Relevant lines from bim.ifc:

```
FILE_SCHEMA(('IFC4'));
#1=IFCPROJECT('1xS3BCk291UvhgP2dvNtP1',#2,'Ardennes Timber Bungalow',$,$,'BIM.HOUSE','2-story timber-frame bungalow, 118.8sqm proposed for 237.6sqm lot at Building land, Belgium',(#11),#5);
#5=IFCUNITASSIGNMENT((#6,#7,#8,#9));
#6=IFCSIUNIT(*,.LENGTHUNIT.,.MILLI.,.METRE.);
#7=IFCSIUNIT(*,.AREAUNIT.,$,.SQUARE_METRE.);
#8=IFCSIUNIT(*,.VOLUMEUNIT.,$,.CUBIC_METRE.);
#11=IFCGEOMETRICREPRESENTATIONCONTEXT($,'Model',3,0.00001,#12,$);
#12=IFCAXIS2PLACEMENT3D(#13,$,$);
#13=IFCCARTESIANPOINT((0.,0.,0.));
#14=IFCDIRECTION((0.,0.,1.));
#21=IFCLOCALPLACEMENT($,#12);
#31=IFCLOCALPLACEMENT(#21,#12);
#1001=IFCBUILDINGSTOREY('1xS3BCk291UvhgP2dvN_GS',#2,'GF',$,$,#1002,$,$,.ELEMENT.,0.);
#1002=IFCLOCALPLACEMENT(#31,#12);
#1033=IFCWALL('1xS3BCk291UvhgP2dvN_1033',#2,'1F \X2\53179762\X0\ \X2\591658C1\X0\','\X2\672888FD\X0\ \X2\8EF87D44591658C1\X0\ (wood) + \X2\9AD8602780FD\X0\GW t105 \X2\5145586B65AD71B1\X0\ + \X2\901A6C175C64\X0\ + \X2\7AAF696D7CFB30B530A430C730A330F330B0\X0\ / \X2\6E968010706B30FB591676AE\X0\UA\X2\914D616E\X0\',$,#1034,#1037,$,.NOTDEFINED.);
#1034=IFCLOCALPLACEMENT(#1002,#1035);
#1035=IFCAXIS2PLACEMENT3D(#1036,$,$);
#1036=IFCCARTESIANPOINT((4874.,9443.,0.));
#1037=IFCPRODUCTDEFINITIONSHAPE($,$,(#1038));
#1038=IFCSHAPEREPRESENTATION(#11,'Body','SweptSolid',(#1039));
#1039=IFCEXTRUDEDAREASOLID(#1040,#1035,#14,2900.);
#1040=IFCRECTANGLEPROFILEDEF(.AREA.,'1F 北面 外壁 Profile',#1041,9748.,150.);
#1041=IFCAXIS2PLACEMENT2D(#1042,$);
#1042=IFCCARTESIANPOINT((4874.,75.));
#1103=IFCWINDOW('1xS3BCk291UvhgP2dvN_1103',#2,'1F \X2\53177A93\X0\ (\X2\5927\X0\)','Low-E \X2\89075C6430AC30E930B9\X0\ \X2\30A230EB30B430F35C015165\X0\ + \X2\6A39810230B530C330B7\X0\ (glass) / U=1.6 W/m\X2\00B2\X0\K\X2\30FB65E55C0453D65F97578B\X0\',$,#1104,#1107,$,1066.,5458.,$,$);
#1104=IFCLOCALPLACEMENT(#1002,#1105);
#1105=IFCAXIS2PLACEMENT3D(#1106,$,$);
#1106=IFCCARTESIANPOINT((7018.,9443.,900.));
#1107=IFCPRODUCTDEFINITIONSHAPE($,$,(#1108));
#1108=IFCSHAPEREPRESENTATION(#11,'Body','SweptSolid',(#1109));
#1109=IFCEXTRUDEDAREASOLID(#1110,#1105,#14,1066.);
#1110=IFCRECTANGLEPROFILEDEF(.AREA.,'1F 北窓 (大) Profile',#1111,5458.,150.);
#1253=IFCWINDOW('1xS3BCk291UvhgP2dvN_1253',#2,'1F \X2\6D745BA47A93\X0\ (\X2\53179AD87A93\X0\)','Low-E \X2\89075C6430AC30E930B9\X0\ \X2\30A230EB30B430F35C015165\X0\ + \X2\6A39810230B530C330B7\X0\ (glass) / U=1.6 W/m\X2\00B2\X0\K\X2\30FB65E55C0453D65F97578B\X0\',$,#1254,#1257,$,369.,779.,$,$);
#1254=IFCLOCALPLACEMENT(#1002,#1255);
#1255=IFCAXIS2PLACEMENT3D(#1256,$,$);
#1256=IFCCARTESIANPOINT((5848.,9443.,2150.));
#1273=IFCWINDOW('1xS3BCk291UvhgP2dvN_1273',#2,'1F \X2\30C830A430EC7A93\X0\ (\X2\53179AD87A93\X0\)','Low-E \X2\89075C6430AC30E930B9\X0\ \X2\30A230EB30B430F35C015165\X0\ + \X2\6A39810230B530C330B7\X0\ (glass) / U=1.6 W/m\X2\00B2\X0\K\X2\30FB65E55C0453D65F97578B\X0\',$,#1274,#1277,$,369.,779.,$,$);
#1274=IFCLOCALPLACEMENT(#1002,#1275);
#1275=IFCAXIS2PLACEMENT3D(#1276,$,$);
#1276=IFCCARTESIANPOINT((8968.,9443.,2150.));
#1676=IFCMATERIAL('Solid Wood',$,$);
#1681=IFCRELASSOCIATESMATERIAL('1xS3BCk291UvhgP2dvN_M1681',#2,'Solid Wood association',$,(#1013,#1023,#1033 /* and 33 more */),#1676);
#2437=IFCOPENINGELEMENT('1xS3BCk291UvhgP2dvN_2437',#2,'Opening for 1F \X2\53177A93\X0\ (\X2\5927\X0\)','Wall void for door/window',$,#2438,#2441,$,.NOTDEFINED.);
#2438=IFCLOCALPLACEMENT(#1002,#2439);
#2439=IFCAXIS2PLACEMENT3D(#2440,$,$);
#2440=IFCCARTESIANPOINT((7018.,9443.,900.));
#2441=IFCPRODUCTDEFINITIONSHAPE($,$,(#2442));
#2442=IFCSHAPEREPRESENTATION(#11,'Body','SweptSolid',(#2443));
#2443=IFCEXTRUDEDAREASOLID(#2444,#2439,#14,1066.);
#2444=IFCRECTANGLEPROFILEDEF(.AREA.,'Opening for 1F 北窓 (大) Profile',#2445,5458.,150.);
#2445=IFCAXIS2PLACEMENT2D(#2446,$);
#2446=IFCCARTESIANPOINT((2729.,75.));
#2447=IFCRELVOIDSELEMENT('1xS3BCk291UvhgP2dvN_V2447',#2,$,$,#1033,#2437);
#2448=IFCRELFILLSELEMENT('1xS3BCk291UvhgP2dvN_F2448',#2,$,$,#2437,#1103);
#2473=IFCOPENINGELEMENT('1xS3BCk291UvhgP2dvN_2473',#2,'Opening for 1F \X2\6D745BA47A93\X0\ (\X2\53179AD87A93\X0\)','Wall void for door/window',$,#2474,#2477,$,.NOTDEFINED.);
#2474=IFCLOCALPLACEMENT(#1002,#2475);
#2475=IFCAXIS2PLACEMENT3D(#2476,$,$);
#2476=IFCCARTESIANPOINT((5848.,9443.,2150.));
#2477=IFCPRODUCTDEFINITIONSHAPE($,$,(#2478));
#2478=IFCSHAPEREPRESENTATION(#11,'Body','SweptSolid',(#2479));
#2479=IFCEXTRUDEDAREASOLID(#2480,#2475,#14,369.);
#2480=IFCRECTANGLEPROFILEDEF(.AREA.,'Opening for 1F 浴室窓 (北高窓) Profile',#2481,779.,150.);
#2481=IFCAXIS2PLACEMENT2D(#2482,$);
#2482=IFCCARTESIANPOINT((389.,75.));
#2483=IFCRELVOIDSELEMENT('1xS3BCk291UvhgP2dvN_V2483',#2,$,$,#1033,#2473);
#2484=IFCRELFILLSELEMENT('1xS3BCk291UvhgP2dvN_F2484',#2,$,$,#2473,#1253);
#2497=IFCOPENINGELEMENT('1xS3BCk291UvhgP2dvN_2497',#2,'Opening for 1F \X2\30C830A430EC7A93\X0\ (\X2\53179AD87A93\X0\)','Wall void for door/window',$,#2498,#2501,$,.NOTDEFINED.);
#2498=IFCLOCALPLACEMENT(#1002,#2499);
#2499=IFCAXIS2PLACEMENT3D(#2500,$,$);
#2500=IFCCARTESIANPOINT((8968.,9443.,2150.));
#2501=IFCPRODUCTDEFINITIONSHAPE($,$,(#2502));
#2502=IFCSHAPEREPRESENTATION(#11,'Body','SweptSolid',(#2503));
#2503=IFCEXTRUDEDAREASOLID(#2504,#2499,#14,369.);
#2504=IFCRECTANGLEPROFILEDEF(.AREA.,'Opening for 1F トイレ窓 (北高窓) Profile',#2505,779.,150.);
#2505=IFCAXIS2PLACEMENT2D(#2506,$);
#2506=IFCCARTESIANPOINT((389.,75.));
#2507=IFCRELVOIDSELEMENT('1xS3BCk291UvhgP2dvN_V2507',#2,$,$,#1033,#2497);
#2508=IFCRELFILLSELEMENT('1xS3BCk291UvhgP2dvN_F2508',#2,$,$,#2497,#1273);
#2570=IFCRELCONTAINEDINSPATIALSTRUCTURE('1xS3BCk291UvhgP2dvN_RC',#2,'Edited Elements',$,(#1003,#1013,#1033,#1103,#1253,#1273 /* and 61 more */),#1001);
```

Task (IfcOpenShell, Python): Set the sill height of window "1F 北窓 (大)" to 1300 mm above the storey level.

```python
import numpy as np
import ifcopenshell
import ifcopenshell.api.geometry
import ifcopenshell.geom
import ifcopenshell.util.element
import ifcopenshell.util.placement
import ifcopenshell.util.shape
import ifcopenshell.util.unit

model = ifcopenshell.open("bim.ifc")
unit_scale = ifcopenshell.util.unit.calculate_unit_scale(model)

window = model.by_id(1103)
opening = window.FillsVoids[0].RelatingOpeningElement
storey = ifcopenshell.util.element.get_container(window, ifc_class="IfcBuildingStorey")
level = ifcopenshell.util.placement.get_local_placement(storey.ObjectPlacement)[2, 3]

# The opening's origin need not be at the sill, so measure its lowest point.
shape = ifcopenshell.geom.create_shape(ifcopenshell.geom.settings(), opening)
bottom = ifcopenshell.util.shape.get_shape_bottom_elevation(shape, shape.geometry) / unit_scale
dz = level + 1300.0 - bottom

shift = np.array([0.0, 0.0, dz])
# The window is not placed relative to its opening, so move both.
for product in (opening, window):
    matrix = ifcopenshell.util.placement.get_local_placement(product.ObjectPlacement)
    matrix[:3, 3] += shift
    ifcopenshell.api.geometry.edit_object_placement(model, product=product, matrix=matrix, is_si=False)

print(f"moved by {dz * unit_scale:+.3f} m")

model.write("bim_updated.ifc")
```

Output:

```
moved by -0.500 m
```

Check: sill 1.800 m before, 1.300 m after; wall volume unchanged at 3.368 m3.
